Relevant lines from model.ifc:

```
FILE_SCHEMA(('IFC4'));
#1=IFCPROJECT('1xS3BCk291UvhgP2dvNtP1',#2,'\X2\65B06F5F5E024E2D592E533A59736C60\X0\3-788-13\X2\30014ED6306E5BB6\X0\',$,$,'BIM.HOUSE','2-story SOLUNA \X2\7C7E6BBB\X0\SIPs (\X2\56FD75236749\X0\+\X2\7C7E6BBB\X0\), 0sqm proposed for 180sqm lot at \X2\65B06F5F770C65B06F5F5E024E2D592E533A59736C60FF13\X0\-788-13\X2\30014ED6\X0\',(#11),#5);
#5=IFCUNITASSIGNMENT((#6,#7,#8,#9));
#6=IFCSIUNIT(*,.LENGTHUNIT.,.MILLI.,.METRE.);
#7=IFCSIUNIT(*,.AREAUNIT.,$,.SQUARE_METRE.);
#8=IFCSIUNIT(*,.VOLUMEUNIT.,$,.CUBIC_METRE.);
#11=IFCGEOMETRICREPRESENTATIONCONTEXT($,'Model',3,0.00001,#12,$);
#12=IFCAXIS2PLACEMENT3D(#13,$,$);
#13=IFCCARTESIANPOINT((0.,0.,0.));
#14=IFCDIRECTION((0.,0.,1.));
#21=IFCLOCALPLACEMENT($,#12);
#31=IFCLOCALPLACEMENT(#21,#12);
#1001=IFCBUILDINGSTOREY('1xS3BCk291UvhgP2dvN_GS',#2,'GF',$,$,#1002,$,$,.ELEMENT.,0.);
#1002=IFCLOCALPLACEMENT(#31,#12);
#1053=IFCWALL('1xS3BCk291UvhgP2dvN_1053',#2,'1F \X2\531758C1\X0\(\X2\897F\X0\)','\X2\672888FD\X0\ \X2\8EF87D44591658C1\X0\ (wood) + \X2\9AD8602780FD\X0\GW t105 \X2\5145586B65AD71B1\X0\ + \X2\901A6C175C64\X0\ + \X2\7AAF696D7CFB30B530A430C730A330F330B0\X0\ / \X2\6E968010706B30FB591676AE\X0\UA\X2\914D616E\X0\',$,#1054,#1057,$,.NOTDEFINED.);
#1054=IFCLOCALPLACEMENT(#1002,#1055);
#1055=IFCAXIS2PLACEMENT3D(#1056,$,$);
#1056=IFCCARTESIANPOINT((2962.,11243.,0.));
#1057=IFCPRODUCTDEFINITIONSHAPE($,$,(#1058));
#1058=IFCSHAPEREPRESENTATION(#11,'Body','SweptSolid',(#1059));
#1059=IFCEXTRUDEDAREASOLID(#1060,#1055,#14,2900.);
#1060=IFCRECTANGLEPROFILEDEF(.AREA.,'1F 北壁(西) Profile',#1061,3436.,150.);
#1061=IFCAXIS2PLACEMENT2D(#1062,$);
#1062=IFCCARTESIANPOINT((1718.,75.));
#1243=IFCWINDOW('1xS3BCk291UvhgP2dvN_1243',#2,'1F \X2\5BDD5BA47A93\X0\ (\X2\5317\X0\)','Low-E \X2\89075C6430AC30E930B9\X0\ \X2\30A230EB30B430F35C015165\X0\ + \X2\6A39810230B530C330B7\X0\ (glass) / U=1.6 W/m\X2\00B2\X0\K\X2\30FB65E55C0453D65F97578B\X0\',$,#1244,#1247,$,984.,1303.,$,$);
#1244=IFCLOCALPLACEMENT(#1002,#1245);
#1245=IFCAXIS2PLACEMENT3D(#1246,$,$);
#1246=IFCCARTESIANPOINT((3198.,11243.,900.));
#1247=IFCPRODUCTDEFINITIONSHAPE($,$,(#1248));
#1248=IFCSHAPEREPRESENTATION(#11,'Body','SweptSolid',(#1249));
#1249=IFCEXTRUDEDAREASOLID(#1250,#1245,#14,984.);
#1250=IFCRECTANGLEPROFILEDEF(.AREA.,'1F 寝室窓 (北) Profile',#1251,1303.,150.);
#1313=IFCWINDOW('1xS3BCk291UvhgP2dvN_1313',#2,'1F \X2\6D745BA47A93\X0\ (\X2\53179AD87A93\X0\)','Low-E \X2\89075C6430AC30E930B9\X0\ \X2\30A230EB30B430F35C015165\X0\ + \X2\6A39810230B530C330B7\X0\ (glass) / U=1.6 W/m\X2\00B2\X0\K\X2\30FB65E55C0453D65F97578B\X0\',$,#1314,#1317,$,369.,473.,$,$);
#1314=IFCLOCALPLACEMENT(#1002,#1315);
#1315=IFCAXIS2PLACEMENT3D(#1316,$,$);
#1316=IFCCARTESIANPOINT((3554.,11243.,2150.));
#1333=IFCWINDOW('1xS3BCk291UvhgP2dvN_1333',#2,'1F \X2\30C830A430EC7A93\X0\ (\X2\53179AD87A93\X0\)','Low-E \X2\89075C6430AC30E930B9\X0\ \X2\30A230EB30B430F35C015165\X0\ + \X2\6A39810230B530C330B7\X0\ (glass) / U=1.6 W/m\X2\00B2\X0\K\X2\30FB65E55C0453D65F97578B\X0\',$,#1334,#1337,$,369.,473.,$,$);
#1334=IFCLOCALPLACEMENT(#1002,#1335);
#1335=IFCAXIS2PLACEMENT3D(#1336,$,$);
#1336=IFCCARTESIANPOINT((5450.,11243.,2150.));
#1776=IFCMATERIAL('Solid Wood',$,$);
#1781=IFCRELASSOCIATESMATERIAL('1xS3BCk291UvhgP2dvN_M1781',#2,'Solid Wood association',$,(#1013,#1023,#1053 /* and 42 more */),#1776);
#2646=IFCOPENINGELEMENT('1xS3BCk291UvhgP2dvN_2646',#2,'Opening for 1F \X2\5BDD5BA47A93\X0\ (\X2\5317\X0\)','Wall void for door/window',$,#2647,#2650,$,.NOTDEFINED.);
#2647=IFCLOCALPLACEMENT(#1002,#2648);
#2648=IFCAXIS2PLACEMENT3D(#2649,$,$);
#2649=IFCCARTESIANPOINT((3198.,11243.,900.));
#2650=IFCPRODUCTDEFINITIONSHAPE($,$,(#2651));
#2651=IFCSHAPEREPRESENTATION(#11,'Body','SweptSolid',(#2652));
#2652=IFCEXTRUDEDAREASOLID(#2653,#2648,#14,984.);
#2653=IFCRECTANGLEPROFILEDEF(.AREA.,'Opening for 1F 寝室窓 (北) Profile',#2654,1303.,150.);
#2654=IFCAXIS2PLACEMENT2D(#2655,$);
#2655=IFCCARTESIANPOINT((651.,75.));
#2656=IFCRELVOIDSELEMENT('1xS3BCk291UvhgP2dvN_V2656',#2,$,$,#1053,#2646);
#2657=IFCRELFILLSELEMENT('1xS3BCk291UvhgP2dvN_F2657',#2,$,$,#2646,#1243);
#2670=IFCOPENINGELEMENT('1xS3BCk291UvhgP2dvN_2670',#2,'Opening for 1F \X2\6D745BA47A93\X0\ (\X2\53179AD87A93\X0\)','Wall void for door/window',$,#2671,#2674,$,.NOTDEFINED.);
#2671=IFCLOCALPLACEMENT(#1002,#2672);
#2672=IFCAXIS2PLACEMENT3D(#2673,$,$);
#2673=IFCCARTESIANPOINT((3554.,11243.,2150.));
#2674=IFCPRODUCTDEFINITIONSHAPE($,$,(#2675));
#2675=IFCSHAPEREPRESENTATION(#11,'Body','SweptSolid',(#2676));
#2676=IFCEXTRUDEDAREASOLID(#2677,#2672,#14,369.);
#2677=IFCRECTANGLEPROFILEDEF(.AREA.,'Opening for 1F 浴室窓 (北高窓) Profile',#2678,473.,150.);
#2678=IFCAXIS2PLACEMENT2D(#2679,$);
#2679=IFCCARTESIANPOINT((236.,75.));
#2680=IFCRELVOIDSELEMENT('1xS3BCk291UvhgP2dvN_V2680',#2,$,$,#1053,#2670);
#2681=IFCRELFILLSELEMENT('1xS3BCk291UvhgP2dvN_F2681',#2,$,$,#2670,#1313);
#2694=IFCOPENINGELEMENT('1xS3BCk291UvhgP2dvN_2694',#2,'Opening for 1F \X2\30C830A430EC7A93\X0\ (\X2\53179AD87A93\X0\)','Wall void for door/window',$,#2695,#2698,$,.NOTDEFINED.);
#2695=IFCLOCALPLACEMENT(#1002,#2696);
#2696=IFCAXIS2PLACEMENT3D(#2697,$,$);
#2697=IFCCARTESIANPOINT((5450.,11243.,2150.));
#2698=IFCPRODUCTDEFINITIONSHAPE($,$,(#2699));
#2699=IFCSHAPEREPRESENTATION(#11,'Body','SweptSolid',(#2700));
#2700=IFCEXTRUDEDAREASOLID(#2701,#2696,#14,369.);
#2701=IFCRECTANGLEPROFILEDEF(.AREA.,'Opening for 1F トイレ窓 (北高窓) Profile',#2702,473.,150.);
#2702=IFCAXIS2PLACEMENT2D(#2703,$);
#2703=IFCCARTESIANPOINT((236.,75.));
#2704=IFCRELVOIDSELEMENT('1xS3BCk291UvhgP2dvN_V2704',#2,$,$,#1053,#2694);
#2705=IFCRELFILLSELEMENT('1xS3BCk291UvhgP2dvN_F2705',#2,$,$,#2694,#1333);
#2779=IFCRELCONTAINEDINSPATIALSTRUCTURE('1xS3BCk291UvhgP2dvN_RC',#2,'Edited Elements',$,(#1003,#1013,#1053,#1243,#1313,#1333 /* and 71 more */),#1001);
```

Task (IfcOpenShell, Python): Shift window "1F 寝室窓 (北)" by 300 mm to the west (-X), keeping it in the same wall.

```python
import ifcopenshell
import ifcopenshell.api.geometry
import ifcopenshell.util.placement

model = ifcopenshell.open("model.ifc")

window = model.by_id(1243)
opening = window.FillsVoids[0].RelatingOpeningElement
wall = opening.VoidsElements[0].RelatingBuildingElement

wall_matrix = ifcopenshell.util.placement.get_local_placement(wall.ObjectPlacement)
shift = wall_matrix[:3, 0] * -300.0
before = ifcopenshell.util.placement.get_local_placement(window.ObjectPlacement)[:3, 3].copy()

# The window is not placed relative to its opening, so move both.
for product in (opening, window):
    matrix = ifcopenshell.util.placement.get_local_placement(product.ObjectPlacement)
    matrix[:3, 3] += shift
    ifcopenshell.api.geometry.edit_object_placement(model, product=product, matrix=matrix, is_si=False)

after = ifcopenshell.util.placement.get_local_placement(window.ObjectPlacement)[:3, 3]
print("window moved by", (after - before).round(3) + 0.0)

model.write("model_edited.ifc")
```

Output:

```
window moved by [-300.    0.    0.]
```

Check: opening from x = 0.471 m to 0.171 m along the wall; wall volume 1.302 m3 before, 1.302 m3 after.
